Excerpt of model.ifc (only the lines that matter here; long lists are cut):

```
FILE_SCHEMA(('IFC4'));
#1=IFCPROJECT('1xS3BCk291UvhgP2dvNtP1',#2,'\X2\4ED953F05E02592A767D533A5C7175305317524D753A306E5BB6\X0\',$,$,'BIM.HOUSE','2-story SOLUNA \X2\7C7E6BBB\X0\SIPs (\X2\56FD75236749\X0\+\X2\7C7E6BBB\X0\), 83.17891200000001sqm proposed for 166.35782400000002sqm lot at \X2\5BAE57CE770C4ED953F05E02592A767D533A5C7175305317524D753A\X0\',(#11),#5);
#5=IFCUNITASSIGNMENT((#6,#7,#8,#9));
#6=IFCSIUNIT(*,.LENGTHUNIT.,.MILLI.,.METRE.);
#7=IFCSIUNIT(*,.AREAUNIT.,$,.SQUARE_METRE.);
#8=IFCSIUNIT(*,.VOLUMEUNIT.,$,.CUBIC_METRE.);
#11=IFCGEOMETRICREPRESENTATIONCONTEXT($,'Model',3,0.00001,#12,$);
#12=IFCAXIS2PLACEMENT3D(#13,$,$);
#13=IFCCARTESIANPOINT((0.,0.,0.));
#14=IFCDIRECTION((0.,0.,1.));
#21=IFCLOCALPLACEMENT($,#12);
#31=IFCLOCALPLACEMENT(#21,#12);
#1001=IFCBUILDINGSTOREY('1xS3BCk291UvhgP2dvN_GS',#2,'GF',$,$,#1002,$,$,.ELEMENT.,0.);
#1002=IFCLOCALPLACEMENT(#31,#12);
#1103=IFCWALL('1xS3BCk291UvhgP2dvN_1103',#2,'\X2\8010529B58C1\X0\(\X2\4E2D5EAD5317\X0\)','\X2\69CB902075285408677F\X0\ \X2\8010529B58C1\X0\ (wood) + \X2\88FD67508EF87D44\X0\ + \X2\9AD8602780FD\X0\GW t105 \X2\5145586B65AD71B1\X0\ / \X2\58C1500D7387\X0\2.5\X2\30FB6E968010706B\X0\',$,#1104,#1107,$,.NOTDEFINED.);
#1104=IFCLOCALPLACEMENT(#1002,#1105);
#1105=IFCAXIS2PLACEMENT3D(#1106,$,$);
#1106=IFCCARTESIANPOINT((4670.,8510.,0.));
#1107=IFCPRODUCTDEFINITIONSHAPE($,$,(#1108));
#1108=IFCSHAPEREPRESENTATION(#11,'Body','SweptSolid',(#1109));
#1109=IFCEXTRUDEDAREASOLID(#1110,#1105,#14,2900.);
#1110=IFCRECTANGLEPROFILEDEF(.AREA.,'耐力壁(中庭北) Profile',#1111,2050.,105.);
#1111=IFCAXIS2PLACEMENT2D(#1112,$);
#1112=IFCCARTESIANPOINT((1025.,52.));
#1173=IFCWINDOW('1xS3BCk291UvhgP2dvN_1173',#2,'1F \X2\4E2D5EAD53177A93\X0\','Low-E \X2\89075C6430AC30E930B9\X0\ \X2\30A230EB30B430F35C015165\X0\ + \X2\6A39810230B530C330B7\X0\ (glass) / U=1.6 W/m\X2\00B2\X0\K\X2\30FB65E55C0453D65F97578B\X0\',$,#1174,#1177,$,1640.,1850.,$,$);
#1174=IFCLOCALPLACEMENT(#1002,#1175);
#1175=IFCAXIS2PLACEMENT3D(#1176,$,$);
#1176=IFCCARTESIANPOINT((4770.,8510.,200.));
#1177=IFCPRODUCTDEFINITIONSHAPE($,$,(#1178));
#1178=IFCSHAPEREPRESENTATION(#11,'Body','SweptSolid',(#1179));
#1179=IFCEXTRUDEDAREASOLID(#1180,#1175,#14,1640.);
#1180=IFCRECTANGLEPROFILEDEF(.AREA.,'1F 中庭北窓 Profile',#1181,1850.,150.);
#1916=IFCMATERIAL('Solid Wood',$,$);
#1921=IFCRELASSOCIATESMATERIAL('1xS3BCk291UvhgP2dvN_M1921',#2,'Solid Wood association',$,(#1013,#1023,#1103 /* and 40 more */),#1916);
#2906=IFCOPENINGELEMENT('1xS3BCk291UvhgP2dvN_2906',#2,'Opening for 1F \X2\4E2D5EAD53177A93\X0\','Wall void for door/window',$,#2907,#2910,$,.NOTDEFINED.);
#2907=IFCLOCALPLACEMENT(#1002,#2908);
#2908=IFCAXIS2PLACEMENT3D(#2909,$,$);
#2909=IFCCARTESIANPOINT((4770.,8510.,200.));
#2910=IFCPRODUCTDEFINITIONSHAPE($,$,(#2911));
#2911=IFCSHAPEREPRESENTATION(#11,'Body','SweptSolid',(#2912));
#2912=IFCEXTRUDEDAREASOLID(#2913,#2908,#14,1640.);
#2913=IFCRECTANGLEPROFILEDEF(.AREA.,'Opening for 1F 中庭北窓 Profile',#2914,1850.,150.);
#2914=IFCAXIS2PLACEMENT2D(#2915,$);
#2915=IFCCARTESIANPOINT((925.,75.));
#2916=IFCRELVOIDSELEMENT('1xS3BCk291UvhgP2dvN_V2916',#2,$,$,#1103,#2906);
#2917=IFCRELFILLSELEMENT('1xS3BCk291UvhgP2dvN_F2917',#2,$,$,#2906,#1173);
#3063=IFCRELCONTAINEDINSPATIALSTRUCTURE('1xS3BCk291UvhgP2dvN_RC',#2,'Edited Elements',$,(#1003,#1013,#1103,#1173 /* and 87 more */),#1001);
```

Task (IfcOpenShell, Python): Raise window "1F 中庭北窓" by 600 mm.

```python
import numpy as np
import ifcopenshell
import ifcopenshell.api.geometry
import ifcopenshell.util.placement
import ifcopenshell.util.unit

model = ifcopenshell.open("model.ifc")
unit_scale = ifcopenshell.util.unit.calculate_unit_scale(model)

window = model.by_id(1173)
opening = window.FillsVoids[0].RelatingOpeningElement
dz = 600.0

shift = np.array([0.0, 0.0, dz])
# The window is not placed relative to its opening, so move both.
for product in (opening, window):
    matrix = ifcopenshell.util.placement.get_local_placement(product.ObjectPlacement)
    matrix[:3, 3] += shift
    ifcopenshell.api.geometry.edit_object_placement(model, product=product, matrix=matrix, is_si=False)

print(f"moved by {dz * unit_scale:+.3f} m")

model.write("model_updated.ifc")
```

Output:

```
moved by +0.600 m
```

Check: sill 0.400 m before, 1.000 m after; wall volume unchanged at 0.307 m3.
